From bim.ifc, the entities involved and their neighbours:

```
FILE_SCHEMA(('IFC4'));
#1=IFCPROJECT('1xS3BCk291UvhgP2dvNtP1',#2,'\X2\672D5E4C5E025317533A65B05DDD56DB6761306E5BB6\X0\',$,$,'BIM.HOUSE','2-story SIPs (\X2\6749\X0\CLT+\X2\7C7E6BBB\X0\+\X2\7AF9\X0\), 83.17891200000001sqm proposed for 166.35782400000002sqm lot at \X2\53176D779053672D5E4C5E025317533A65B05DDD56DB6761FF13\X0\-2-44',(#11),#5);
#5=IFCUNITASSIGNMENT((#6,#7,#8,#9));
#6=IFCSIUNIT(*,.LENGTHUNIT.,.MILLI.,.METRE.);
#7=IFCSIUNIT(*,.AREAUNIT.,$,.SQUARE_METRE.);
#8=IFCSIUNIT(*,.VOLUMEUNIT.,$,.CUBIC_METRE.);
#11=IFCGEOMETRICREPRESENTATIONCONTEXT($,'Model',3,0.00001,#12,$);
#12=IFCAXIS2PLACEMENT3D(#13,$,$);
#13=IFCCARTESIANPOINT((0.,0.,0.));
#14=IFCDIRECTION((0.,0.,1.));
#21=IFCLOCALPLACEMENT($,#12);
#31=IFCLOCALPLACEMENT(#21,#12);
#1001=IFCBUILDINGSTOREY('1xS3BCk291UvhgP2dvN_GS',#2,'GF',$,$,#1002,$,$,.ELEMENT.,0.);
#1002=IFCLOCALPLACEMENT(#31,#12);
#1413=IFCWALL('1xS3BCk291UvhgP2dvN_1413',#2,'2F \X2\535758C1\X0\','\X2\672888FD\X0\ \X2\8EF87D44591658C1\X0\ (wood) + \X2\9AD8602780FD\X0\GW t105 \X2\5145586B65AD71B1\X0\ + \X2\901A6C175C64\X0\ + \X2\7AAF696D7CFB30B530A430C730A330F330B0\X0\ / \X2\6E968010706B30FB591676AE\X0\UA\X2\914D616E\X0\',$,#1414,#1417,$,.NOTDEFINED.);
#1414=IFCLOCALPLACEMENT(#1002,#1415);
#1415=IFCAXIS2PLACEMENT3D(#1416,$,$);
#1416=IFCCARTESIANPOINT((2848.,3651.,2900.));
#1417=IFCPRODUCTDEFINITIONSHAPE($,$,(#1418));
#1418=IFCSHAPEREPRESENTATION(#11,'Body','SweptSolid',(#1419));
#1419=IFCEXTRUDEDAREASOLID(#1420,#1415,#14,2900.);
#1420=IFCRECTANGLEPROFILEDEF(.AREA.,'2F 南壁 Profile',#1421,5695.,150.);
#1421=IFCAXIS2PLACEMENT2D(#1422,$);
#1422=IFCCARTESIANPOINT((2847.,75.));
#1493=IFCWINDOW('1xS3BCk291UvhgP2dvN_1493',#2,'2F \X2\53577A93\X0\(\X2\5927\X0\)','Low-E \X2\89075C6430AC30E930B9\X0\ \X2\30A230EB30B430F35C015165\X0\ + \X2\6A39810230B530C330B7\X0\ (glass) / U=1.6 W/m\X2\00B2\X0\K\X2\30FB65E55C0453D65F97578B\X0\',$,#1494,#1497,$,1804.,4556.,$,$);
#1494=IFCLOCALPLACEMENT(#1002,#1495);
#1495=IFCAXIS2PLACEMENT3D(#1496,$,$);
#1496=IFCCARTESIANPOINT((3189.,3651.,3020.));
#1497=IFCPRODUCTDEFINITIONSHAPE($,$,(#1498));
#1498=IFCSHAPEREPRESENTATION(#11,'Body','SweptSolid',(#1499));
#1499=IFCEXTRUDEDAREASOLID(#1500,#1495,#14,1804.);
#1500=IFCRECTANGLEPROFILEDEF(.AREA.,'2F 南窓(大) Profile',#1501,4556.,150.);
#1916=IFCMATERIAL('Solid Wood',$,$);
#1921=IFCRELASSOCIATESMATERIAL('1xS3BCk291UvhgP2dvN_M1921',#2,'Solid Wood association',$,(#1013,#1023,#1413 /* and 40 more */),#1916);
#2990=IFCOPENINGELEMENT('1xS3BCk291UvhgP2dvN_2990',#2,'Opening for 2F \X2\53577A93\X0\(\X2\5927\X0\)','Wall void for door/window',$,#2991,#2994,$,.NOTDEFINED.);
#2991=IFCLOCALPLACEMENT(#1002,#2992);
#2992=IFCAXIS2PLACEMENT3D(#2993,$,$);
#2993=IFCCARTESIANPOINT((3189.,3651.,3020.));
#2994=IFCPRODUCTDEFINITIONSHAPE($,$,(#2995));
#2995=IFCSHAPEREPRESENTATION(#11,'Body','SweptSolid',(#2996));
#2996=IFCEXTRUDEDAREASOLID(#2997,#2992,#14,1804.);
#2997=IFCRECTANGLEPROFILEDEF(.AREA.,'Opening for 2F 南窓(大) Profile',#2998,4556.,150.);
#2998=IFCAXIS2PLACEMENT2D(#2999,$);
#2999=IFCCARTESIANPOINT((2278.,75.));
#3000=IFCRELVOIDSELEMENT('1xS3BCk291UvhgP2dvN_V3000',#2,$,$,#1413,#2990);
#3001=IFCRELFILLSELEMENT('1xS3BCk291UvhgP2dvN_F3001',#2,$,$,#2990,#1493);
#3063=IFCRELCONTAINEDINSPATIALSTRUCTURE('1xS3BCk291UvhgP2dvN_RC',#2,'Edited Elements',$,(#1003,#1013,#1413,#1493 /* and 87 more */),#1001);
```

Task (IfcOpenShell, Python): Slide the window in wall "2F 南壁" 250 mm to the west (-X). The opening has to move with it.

```python
import ifcopenshell
import ifcopenshell.api.geometry
import ifcopenshell.util.placement

model = ifcopenshell.open("bim.ifc")

window = model.by_guid("1xS3BCk291UvhgP2dvN_1493")
opening = window.FillsVoids[0].RelatingOpeningElement
wall = opening.VoidsElements[0].RelatingBuildingElement

wall_matrix = ifcopenshell.util.placement.get_local_placement(wall.ObjectPlacement)
shift = wall_matrix[:3, 0] * -250.0
before = ifcopenshell.util.placement.get_local_placement(window.ObjectPlacement)[:3, 3].copy()

# The window is not placed relative to its opening, so move both.
for product in (opening, window):
    matrix = ifcopenshell.util.placement.get_local_placement(product.ObjectPlacement)
    matrix[:3, 3] += shift
    ifcopenshell.api.geometry.edit_object_placement(model, product=product, matrix=matrix, is_si=False)

after = ifcopenshell.util.placement.get_local_placement(window.ObjectPlacement)[:3, 3]
print("window moved by", (after - before).round(3) + 0.0)

model.write("bim-out.ifc")
```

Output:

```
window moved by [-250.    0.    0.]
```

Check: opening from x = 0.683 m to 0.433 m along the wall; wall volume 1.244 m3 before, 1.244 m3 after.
